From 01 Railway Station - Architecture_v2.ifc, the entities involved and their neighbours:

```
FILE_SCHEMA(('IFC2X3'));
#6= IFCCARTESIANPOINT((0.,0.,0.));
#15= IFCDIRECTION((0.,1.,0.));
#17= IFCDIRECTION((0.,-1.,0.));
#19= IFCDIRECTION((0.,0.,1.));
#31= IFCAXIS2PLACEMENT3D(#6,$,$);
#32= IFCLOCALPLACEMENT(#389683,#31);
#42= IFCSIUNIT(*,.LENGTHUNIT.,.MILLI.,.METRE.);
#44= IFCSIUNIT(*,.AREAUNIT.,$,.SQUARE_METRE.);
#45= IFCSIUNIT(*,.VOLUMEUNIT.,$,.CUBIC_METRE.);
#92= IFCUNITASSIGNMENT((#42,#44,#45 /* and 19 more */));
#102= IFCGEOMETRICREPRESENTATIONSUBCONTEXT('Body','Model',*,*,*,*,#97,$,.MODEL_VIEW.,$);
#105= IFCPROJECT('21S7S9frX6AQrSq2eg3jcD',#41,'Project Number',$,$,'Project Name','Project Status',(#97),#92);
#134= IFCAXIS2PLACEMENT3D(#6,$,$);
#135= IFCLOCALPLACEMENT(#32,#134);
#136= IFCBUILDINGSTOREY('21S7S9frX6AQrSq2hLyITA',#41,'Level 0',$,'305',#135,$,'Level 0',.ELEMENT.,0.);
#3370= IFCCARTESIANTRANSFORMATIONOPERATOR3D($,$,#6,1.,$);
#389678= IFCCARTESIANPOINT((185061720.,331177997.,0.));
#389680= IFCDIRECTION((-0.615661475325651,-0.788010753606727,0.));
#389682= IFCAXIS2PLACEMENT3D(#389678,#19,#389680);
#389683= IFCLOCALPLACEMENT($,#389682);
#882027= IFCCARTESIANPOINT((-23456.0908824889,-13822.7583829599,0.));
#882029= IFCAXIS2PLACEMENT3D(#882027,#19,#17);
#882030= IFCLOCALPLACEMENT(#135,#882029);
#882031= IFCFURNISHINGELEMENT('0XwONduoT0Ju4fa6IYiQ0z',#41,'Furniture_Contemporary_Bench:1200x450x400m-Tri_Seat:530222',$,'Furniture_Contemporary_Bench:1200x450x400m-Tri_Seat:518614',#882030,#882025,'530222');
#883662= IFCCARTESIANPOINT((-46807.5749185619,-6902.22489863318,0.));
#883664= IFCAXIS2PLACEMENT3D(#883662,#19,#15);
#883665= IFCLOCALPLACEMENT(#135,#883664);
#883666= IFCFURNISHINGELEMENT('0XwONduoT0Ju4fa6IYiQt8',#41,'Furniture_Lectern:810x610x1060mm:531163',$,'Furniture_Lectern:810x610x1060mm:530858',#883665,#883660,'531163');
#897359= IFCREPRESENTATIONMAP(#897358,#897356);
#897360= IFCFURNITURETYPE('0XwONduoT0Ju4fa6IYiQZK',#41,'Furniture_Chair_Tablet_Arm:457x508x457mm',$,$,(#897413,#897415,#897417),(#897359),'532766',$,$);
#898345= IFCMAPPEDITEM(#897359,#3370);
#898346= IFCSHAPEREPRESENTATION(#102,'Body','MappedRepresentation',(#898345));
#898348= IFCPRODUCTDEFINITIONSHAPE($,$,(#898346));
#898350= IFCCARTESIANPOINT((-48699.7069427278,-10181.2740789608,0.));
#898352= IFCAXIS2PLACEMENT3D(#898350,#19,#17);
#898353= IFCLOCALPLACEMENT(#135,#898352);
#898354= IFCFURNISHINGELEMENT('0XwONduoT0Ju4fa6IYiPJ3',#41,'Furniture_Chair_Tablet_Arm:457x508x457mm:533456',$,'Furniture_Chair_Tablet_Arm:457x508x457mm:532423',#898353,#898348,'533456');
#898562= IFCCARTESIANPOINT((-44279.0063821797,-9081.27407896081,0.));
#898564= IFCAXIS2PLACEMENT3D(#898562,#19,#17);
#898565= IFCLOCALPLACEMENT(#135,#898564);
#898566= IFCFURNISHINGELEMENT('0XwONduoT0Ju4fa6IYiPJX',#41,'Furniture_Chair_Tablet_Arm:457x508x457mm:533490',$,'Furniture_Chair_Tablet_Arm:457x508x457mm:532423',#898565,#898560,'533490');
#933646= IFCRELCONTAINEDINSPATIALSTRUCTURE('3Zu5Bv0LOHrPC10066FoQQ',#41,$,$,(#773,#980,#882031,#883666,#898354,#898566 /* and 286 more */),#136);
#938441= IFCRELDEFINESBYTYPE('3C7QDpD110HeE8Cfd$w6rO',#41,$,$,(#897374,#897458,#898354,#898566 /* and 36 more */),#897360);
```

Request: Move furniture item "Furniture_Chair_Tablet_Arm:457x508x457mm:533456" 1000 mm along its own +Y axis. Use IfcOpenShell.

```python
import ifcopenshell
import ifcopenshell.api.geometry
import ifcopenshell.util.placement

model = ifcopenshell.open("01 Railway Station - Architecture_v2.ifc")

item = model.by_guid("0XwONduoT0Ju4fa6IYiPJ3")
matrix = ifcopenshell.util.placement.get_local_placement(item.ObjectPlacement)
matrix[:3, 3] += matrix[:3, 1] * 1000.0
ifcopenshell.api.geometry.edit_object_placement(model, product=item, matrix=matrix, is_si=False)

print(ifcopenshell.util.placement.get_local_placement(item.ObjectPlacement).round(3) + 0.0)

model.write("01 Railway Station - Architecture_v2_v2.ifc")
```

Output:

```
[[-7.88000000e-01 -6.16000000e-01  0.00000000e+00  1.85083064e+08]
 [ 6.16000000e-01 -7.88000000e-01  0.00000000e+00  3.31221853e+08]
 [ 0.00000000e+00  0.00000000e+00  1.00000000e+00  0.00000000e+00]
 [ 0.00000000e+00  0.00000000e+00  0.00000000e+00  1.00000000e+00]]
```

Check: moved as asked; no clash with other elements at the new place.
